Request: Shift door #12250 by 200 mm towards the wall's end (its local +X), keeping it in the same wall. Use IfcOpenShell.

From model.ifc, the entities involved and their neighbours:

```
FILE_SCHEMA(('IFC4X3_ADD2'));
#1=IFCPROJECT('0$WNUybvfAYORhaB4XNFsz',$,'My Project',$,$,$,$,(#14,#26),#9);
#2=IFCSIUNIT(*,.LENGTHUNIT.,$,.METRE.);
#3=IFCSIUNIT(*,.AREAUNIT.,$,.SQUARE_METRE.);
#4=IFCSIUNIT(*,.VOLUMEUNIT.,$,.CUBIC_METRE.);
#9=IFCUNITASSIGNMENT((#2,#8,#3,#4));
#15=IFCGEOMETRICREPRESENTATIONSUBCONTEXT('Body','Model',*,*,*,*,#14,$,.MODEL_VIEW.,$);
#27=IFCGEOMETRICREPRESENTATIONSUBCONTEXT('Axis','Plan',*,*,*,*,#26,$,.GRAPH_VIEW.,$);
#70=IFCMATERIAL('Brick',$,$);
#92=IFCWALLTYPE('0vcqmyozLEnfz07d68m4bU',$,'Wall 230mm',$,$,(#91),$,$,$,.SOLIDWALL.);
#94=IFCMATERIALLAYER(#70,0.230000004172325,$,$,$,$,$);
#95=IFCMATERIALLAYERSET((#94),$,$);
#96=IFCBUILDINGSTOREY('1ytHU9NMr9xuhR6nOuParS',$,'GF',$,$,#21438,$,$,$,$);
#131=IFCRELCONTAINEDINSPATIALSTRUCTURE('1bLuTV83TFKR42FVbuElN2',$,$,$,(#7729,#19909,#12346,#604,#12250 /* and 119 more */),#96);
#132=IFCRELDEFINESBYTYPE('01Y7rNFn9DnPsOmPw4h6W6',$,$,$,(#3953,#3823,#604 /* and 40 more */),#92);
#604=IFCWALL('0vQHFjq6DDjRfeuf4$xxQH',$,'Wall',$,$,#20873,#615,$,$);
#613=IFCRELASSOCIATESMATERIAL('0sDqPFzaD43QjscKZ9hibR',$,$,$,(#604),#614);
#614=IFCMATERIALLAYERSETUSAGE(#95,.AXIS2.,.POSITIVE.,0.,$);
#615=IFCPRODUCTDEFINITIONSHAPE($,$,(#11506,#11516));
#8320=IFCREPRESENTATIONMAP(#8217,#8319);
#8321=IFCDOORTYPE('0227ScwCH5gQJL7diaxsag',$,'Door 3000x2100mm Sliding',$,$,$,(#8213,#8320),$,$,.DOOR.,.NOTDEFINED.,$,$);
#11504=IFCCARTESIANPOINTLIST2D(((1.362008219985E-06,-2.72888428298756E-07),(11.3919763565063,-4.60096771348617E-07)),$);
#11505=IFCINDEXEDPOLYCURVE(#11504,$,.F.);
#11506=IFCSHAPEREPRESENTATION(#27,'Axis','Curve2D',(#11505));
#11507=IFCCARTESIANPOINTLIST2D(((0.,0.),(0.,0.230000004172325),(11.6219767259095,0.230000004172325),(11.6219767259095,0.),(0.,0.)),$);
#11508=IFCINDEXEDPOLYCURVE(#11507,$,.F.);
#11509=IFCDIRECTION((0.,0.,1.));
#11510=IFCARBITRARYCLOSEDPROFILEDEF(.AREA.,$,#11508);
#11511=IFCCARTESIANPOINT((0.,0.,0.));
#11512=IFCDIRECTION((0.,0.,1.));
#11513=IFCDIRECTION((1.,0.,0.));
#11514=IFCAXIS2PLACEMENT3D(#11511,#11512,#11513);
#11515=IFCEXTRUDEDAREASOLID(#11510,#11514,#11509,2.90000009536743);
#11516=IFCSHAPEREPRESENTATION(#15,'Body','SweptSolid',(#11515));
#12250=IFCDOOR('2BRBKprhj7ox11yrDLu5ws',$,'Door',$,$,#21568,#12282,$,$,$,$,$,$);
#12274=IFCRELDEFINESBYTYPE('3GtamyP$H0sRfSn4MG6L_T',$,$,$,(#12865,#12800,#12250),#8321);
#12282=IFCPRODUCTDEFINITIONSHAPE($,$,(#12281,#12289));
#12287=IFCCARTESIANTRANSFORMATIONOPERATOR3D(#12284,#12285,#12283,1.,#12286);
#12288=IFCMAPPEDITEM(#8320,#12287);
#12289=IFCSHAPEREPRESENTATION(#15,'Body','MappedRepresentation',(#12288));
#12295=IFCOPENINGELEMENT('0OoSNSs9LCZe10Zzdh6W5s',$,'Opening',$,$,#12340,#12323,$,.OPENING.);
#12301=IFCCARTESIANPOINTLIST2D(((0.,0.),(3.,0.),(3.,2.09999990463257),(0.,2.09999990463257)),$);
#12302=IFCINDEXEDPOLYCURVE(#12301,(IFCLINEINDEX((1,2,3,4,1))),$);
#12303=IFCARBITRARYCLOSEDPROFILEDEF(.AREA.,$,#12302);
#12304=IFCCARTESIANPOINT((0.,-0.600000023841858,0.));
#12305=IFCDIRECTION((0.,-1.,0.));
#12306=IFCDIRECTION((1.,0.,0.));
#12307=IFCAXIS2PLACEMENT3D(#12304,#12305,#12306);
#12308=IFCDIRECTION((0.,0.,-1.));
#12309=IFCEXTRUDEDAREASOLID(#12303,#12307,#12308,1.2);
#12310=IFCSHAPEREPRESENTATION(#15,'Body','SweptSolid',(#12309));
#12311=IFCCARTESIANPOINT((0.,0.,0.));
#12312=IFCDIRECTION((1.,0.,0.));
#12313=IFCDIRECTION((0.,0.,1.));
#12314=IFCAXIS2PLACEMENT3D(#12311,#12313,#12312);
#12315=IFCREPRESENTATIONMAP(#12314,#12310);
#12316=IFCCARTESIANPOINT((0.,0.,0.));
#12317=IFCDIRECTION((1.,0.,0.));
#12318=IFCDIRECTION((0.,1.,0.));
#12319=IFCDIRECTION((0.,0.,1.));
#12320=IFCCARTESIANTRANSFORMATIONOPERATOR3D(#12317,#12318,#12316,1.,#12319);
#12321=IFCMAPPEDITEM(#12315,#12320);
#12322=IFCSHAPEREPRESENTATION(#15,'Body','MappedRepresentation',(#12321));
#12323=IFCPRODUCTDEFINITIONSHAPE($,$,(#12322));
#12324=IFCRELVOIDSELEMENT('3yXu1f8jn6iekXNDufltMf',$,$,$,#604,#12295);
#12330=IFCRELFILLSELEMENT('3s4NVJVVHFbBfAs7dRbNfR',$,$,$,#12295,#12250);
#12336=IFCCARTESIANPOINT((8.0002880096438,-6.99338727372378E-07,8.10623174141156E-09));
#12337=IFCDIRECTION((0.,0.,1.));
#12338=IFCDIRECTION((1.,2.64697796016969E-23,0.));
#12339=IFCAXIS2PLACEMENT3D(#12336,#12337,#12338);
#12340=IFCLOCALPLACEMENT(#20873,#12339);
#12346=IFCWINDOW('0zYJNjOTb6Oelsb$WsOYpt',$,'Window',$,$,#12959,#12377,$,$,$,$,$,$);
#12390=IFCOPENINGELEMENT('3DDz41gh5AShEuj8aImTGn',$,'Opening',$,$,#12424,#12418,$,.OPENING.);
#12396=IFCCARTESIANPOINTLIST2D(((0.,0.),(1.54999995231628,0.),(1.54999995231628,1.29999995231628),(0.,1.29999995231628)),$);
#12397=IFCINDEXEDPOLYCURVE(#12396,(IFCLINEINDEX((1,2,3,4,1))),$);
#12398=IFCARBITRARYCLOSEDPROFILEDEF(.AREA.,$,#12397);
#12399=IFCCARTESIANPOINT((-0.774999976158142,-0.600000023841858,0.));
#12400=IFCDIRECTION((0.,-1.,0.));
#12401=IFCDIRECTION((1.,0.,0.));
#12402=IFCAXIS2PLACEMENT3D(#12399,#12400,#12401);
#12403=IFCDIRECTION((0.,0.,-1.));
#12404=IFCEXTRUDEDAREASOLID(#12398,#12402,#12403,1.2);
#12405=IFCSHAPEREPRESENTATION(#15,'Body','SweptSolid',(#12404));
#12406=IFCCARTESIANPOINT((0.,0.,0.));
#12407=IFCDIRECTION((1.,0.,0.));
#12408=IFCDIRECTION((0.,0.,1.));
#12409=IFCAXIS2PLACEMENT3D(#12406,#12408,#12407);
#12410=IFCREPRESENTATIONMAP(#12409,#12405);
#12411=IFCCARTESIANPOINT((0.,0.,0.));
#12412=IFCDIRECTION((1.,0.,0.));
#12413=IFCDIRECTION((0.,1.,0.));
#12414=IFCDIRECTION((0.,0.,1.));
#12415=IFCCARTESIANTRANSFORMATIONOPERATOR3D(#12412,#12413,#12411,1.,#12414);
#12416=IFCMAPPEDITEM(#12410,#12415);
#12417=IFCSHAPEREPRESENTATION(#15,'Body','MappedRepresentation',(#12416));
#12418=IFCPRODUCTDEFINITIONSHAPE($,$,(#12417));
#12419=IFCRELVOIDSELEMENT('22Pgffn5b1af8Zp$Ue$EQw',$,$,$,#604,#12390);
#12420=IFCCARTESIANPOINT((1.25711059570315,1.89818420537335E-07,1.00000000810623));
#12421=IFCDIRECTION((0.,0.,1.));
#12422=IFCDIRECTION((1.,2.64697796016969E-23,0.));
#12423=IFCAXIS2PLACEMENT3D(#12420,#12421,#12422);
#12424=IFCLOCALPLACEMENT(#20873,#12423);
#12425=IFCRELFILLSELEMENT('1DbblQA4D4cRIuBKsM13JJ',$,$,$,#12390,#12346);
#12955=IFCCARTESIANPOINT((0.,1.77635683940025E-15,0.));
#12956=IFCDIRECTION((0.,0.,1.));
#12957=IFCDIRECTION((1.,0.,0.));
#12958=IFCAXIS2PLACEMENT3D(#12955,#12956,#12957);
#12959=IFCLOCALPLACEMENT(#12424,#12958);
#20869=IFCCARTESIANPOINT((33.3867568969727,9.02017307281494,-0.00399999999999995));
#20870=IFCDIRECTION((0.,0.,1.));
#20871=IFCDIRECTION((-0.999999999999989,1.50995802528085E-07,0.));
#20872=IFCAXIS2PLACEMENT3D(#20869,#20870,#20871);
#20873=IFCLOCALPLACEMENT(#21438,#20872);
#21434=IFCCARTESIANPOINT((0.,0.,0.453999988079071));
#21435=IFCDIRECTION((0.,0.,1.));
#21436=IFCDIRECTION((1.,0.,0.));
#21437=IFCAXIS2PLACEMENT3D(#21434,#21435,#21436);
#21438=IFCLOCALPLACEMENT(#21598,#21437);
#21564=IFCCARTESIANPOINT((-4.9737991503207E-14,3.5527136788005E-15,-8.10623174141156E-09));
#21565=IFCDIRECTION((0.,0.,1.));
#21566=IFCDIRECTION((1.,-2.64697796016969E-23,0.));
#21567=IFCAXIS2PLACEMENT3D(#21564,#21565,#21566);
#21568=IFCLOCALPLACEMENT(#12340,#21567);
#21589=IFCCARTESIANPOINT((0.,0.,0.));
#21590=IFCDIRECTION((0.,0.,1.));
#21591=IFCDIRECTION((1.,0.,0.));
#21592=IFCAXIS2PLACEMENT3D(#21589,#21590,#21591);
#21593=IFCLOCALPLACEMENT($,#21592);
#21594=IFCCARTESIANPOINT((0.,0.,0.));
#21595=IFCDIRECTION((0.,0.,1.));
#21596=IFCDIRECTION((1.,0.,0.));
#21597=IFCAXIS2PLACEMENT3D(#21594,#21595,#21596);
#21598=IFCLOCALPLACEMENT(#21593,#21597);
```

```python
import ifcopenshell
import ifcopenshell.api.geometry
import ifcopenshell.util.placement
import ifcopenshell.util.unit

model = ifcopenshell.open("model.ifc")
unit_scale = ifcopenshell.util.unit.calculate_unit_scale(model)

door = model.by_guid("2BRBKprhj7ox11yrDLu5ws")
opening = door.FillsVoids[0].RelatingOpeningElement
wall = opening.VoidsElements[0].RelatingBuildingElement

wall_matrix = ifcopenshell.util.placement.get_local_placement(wall.ObjectPlacement)
shift = wall_matrix[:3, 0] * 0.2 / unit_scale
before = ifcopenshell.util.placement.get_local_placement(door.ObjectPlacement)[:3, 3].copy()

# The door is placed relative to its opening, so it follows when the opening moves.
matrix = ifcopenshell.util.placement.get_local_placement(opening.ObjectPlacement)
matrix[:3, 3] += shift
ifcopenshell.api.geometry.edit_object_placement(
    model, product=opening, matrix=matrix, is_si=False, should_transform_children=True
)

after = ifcopenshell.util.placement.get_local_placement(door.ObjectPlacement)[:3, 3]
print("door moved by", (after - before).round(3) + 0.0)

model.write("model_v2.ifc")
```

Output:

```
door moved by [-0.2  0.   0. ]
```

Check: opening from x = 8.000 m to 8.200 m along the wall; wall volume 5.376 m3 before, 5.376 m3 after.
